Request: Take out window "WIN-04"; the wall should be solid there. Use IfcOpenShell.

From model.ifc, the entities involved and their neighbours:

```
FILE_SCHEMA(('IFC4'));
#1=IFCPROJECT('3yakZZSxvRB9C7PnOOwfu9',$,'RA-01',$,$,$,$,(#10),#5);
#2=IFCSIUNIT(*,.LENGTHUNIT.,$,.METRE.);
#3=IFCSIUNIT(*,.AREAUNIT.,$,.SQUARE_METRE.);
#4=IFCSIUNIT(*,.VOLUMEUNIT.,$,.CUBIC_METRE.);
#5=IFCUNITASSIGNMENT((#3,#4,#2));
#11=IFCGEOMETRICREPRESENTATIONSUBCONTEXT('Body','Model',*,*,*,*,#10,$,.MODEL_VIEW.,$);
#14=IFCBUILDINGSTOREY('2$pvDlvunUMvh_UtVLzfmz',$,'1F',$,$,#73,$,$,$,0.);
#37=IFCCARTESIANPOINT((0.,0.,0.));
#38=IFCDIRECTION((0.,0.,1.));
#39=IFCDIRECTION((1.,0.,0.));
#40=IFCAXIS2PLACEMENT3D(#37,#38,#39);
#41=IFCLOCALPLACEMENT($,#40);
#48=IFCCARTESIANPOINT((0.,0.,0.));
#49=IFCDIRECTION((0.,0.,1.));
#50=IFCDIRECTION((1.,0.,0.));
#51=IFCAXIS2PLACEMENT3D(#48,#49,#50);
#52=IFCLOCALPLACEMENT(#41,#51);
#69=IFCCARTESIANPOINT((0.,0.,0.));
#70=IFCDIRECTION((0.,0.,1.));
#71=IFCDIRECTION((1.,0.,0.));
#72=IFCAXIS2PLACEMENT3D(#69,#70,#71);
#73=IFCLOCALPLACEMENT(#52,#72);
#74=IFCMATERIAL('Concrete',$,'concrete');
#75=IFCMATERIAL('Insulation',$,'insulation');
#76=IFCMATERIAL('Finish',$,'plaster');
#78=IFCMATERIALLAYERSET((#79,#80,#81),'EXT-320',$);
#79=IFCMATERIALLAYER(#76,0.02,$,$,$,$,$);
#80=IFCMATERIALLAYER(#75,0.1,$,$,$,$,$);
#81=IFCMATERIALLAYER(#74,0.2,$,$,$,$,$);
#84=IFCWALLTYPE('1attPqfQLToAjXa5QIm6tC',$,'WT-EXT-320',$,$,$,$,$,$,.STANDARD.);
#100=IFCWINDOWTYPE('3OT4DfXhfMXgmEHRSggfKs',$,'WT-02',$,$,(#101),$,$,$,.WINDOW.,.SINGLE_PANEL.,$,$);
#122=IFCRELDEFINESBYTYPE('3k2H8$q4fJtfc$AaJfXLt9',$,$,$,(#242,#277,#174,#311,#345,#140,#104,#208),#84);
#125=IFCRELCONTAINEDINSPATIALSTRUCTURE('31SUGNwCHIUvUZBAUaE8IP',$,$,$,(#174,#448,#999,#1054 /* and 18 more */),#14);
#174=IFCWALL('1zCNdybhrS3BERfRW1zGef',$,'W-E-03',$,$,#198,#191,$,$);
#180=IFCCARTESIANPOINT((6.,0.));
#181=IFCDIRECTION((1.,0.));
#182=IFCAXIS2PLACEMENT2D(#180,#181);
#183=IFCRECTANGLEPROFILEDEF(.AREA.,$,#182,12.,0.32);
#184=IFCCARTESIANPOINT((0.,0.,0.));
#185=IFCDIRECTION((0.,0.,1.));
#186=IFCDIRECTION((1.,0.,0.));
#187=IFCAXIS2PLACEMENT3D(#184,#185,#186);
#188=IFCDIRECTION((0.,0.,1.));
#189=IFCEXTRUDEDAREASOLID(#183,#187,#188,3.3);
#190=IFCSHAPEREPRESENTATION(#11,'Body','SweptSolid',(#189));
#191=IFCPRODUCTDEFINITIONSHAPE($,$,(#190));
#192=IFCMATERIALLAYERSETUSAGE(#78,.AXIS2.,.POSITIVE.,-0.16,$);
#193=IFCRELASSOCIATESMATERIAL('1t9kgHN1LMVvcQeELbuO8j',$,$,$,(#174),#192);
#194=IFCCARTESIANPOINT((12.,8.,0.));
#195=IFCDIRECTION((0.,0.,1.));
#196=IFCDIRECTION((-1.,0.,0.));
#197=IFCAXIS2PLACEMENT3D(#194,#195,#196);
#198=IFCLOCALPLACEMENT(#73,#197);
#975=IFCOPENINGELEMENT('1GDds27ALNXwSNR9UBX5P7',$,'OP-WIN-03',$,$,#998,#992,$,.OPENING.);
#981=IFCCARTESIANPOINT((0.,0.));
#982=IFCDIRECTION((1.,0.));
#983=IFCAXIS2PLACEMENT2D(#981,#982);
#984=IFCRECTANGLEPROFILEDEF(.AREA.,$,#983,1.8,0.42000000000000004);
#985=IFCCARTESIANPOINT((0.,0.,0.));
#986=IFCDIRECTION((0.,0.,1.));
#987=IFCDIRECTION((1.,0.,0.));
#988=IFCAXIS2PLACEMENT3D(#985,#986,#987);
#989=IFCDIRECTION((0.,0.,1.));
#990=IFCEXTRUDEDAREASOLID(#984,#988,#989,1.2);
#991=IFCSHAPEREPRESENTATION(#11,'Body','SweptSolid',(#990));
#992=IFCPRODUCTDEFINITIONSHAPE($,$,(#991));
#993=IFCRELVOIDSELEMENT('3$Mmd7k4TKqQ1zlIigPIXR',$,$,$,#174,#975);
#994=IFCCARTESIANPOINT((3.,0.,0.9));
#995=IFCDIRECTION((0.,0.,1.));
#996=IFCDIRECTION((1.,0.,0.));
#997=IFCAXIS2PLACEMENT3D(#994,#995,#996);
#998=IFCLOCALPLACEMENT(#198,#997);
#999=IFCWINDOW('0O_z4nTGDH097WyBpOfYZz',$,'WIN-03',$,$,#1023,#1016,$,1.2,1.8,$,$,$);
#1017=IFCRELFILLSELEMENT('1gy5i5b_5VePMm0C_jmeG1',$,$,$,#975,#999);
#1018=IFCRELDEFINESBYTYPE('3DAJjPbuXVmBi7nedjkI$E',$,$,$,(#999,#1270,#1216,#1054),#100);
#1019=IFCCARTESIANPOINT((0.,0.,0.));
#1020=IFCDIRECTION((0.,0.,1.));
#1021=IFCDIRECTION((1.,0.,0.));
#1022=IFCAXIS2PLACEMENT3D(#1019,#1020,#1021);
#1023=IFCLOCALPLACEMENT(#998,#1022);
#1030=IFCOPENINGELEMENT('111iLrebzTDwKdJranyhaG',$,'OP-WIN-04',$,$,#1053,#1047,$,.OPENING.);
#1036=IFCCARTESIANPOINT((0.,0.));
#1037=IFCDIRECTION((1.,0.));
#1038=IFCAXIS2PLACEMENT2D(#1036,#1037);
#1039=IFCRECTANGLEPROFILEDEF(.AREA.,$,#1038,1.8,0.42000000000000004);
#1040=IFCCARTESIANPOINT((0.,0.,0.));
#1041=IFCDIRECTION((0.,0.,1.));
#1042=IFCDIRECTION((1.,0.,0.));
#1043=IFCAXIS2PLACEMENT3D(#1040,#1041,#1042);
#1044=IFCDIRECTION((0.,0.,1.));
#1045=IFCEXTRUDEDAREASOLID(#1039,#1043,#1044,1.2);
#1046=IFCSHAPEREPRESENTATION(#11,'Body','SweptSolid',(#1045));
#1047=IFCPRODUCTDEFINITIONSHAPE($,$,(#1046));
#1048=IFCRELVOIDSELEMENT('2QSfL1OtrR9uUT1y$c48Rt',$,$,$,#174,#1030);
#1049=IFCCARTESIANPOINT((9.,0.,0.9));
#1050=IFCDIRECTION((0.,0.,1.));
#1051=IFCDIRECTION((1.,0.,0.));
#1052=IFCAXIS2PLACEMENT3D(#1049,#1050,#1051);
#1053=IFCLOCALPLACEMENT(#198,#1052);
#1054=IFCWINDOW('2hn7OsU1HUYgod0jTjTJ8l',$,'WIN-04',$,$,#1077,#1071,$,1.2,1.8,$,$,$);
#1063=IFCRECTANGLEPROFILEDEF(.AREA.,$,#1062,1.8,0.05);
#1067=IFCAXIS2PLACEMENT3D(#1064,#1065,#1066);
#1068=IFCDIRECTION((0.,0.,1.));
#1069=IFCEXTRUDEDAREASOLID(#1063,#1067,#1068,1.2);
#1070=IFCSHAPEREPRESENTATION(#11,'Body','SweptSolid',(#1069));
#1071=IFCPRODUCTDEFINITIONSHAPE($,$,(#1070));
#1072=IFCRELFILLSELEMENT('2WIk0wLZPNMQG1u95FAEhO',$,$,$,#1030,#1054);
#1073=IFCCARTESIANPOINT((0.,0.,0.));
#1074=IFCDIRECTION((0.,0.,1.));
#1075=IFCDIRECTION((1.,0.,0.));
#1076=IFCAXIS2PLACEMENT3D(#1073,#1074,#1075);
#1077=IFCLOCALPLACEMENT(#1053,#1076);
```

```python
import ifcopenshell
import ifcopenshell.api.feature
import ifcopenshell.api.root
import ifcopenshell.geom
import ifcopenshell.util.shape

model = ifcopenshell.open("model.ifc")
settings = ifcopenshell.geom.settings()


def volume(element):
    """Net volume in cubic metres, openings subtracted."""
    shape = ifcopenshell.geom.create_shape(settings, element)
    return ifcopenshell.util.shape.get_volume(shape.geometry)


window = model.by_id(1054)
opening = window.FillsVoids[0].RelatingOpeningElement
wall = opening.VoidsElements[0].RelatingBuildingElement
before = volume(wall)

ifcopenshell.api.root.remove_product(model, product=window)
ifcopenshell.api.feature.remove_feature(model, feature=opening)

after = volume(wall)

print(f"wall volume {before:.3f} -> {after:.3f} m3")

model.write("model_updated.ifc")
```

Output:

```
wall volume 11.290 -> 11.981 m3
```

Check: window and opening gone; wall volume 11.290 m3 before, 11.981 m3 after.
